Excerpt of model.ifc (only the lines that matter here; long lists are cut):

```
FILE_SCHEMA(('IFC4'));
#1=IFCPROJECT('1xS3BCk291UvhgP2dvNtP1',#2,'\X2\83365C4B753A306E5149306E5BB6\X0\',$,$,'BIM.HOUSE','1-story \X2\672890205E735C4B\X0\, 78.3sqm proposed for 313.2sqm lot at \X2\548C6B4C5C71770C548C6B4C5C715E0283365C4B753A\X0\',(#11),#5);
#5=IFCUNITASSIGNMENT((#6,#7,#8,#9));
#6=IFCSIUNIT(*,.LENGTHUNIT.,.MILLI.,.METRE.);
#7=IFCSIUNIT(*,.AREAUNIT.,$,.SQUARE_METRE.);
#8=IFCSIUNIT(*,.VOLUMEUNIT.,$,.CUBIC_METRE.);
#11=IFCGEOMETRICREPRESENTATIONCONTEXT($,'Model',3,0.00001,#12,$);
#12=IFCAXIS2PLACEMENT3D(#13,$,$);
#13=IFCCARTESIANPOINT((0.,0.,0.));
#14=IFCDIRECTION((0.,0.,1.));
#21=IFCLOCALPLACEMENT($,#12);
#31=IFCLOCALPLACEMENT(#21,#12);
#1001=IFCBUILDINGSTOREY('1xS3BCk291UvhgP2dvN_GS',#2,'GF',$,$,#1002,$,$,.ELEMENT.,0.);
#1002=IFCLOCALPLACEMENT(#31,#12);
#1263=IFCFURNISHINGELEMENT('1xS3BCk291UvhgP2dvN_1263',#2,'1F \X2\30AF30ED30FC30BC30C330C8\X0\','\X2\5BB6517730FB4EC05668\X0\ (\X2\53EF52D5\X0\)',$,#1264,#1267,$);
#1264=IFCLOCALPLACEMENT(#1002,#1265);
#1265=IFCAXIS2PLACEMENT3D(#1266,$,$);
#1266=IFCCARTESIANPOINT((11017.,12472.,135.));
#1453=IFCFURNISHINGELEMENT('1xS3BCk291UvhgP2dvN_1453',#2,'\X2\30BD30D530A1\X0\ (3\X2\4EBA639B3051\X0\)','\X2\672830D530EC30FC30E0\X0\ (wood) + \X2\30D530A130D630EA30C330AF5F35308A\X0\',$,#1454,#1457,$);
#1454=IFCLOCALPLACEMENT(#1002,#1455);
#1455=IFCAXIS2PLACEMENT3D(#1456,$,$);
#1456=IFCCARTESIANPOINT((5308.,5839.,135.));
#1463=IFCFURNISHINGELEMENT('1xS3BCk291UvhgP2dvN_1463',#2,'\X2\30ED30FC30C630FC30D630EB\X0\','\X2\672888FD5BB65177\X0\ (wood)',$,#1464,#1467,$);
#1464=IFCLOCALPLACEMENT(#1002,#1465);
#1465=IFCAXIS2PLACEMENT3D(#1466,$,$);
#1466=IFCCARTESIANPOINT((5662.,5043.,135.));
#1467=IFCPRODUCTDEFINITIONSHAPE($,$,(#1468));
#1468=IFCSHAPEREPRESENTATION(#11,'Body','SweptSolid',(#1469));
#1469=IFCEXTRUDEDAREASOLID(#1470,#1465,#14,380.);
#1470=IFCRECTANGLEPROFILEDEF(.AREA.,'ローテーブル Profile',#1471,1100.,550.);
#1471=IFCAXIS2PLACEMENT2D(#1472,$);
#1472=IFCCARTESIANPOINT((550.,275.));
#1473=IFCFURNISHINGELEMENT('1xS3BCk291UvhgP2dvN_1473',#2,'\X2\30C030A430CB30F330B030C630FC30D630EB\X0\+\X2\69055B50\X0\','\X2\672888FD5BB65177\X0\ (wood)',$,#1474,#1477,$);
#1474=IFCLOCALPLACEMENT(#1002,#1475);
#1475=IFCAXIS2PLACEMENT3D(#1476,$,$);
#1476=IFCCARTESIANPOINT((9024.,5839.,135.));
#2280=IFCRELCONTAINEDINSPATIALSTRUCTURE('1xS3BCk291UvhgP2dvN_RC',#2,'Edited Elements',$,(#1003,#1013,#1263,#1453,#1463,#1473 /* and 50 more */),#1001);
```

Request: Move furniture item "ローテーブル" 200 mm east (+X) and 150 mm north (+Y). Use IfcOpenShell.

```python
import ifcopenshell
import ifcopenshell.api.geometry
import ifcopenshell.util.placement

model = ifcopenshell.open("model.ifc")

item = model.by_guid("1xS3BCk291UvhgP2dvN_1463")
matrix = ifcopenshell.util.placement.get_local_placement(item.ObjectPlacement)
matrix[0, 3] += 200.0
matrix[1, 3] += 150.0
ifcopenshell.api.geometry.edit_object_placement(model, product=item, matrix=matrix, is_si=False)

print(ifcopenshell.util.placement.get_local_placement(item.ObjectPlacement).round(3) + 0.0)

model.write("model_v2.ifc")
```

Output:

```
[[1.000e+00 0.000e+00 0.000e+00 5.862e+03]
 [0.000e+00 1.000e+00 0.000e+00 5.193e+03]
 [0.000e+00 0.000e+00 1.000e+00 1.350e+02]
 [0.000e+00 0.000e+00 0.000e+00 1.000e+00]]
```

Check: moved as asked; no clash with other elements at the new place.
